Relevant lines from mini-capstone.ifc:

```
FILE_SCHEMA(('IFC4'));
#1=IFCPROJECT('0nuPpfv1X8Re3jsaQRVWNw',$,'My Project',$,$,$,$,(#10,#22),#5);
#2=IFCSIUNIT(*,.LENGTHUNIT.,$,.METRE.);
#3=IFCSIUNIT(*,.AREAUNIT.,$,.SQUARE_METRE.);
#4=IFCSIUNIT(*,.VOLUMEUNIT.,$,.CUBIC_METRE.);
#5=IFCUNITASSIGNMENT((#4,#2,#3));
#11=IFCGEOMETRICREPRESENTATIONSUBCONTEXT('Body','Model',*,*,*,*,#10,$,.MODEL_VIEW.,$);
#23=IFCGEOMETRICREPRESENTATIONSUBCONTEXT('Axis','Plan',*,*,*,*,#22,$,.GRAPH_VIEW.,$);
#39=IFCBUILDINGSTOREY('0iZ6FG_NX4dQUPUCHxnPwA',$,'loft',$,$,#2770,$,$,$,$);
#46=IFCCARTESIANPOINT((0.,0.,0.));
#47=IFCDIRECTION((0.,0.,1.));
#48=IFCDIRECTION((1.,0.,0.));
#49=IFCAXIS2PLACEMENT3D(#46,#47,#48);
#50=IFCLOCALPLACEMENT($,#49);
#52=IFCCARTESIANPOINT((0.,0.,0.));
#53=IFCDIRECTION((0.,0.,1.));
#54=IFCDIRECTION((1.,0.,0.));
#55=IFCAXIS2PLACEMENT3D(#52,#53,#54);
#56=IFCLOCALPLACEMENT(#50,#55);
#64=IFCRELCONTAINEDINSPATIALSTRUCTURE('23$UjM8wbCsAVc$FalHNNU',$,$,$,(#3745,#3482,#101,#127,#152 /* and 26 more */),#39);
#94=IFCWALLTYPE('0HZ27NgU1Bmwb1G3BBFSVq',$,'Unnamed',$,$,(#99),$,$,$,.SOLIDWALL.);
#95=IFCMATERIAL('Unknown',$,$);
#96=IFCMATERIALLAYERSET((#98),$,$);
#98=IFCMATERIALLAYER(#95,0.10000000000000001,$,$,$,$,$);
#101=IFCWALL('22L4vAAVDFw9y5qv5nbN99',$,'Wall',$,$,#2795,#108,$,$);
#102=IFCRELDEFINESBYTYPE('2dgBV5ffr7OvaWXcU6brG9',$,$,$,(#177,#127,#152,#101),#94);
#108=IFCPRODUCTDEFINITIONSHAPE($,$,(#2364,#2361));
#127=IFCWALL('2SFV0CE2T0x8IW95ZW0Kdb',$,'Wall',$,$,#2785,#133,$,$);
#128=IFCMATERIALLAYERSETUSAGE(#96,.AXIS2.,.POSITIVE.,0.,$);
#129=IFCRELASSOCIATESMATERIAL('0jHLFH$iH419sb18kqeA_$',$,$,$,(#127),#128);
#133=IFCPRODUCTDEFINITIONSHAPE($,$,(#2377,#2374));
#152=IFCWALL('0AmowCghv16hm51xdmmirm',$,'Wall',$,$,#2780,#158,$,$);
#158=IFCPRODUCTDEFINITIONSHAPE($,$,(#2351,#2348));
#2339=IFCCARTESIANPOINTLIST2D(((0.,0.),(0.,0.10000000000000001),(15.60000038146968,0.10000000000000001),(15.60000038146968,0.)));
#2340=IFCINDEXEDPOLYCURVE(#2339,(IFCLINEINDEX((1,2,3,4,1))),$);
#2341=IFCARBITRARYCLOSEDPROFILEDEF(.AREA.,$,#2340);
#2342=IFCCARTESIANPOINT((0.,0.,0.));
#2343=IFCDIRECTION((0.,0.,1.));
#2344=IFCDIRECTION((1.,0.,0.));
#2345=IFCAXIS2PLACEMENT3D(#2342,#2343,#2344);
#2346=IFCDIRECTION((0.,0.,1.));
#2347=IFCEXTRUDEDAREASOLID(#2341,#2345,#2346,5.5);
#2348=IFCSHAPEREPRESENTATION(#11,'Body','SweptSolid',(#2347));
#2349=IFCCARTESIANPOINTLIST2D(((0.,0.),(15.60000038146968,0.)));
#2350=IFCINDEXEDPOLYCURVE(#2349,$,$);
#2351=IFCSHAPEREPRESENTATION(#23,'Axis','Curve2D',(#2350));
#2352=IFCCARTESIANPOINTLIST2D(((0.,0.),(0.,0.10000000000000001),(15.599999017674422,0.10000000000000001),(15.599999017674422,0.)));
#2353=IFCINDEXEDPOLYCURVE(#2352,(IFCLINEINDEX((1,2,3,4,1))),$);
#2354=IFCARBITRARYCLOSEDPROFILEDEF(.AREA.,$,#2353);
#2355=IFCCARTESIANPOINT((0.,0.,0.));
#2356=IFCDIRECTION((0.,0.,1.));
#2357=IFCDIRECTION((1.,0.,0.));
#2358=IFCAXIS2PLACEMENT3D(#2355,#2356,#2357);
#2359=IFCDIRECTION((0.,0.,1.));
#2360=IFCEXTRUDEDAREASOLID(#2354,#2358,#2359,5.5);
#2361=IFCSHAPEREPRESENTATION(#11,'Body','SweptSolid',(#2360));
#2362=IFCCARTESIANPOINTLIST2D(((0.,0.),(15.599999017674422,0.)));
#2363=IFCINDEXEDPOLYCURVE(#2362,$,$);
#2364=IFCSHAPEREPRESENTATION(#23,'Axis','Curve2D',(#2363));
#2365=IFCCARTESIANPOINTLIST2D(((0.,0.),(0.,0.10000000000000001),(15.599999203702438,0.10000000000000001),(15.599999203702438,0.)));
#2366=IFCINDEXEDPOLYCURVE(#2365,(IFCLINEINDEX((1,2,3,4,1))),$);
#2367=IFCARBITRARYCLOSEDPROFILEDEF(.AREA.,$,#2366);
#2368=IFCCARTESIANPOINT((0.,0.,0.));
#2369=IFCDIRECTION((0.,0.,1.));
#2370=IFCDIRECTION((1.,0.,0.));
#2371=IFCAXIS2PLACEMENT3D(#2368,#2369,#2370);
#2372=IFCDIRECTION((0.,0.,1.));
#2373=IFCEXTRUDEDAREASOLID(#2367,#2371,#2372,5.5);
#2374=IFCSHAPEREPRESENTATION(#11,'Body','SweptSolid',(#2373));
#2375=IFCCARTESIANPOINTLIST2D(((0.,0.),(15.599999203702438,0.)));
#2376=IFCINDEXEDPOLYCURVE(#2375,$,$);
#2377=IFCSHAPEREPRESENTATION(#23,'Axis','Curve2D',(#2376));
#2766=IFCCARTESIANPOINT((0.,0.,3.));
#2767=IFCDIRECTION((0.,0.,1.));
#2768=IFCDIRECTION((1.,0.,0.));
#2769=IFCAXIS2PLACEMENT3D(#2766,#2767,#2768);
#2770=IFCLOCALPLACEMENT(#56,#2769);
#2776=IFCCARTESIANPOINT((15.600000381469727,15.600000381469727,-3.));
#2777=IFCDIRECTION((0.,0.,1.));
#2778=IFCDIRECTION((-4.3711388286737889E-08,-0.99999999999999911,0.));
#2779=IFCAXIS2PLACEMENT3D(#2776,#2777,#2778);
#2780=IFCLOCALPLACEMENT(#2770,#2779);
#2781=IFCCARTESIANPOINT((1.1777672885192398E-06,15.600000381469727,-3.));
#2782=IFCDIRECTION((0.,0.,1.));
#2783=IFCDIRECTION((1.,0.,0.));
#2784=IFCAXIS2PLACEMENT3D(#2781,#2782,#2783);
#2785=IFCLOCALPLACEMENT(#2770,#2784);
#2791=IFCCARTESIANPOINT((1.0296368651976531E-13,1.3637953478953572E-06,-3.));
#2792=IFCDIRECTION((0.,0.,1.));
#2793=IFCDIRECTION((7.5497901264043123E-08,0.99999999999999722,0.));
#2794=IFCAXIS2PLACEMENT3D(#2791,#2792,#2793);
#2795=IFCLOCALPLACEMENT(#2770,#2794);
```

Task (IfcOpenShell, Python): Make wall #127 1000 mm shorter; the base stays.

```python
import ifcopenshell
import ifcopenshell.geom
import ifcopenshell.util.representation
import ifcopenshell.util.shape

model = ifcopenshell.open("mini-capstone.ifc")
settings = ifcopenshell.geom.settings()


def volume(element):
    """Net volume in cubic metres, openings subtracted."""
    shape = ifcopenshell.geom.create_shape(settings, element)
    return ifcopenshell.util.shape.get_volume(shape.geometry)


wall = model.by_id(127)
before = volume(wall)

body = ifcopenshell.util.representation.get_representation(wall, "Model", "Body")
solid = body.Items[0]
old_height = solid.Depth
solid.Depth -= 1.0
after = volume(wall)

print(f"height {old_height:g} -> {solid.Depth:g}, volume {before:.3f} -> {after:.3f} m3")

model.write("mini-capstone_edited.ifc")
```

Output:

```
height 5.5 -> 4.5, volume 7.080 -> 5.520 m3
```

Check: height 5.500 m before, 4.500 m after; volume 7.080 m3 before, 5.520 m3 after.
